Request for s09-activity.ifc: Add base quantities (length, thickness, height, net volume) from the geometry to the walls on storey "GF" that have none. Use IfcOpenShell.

First a look at what the model holds.

```python
import ifcopenshell
import ifcopenshell.util.element
import ifcopenshell.util.unit

model = ifcopenshell.open("s09-activity.ifc")
print(model.schema)
for unit_type in ("LENGTHUNIT", "AREAUNIT", "VOLUMEUNIT"):
    print(unit_type, ifcopenshell.util.unit.calculate_unit_scale(model, unit_type))
storey = next(s for s in model.by_type("IfcBuildingStorey") if s.Name == "GF")
walls = [e for e in ifcopenshell.util.element.get_decomposition(storey) if e.is_a("IfcWall")]
for e in sorted(walls, key=lambda e: e.id()):
    print(e.id(), e.is_a(), e.Name, list(ifcopenshell.util.element.get_psets(e, qtos_only=True)), sep=" | ")
```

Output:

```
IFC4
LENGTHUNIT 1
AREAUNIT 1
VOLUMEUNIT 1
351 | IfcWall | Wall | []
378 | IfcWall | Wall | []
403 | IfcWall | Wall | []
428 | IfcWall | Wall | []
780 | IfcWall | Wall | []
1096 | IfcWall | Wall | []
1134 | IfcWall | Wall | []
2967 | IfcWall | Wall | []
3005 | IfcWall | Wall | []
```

```python
import ifcopenshell
import ifcopenshell.api.pset
import ifcopenshell.geom
import ifcopenshell.util.element
import ifcopenshell.util.shape
import ifcopenshell.util.unit

model = ifcopenshell.open("s09-activity.ifc")
unit_scale = ifcopenshell.util.unit.calculate_unit_scale(model)
volume_scale = ifcopenshell.util.unit.calculate_unit_scale(model, "VOLUMEUNIT")
settings = ifcopenshell.geom.settings()

storey = next(s for s in model.by_type("IfcBuildingStorey") if s.Name == "GF")
walls = [e for e in ifcopenshell.util.element.get_decomposition(storey) if e.is_a("IfcWall")]

for e in sorted(walls, key=lambda e: e.id()):
    if ifcopenshell.util.element.get_psets(e, qtos_only=True, should_inherit=False):
        continue
    # Geometry comes back in metres, in the element's own axes.
    shape = ifcopenshell.geom.create_shape(settings, e)
    values = {
        "Length": ifcopenshell.util.shape.get_x(shape.geometry) / unit_scale,
        "Width": ifcopenshell.util.shape.get_y(shape.geometry) / unit_scale,
        "Height": ifcopenshell.util.shape.get_z(shape.geometry) / unit_scale,
        "NetVolume": ifcopenshell.util.shape.get_volume(shape.geometry) / volume_scale,
    }
    qto = ifcopenshell.api.pset.add_qto(model, product=e, name="Qto_WallBaseQuantities")
    ifcopenshell.api.pset.edit_qto(model, qto=qto, properties=values)
    print(e.id(), {k: round(v, 3) for k, v in values.items()})

model.write("s09-activity-out.ifc")
```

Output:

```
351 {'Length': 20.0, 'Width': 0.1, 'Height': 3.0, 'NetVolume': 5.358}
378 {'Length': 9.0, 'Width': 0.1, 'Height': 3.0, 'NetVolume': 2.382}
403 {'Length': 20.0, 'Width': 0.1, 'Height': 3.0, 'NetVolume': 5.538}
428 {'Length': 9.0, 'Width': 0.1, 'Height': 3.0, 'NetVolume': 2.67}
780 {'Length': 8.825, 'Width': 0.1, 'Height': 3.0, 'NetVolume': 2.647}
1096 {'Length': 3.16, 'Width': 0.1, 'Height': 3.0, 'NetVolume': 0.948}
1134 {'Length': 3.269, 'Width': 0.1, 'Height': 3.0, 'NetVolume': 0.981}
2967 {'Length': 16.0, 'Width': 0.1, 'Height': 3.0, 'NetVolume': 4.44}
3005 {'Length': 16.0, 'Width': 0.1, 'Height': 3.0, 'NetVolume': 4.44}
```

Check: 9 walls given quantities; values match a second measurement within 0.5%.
